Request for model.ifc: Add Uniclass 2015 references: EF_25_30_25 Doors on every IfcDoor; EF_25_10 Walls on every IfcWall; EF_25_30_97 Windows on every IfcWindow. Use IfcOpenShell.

First a look at what the model holds.

```python
import ifcopenshell

model = ifcopenshell.open("model.ifc")
print(model.schema)
print("classifications:", [c.Name for c in model.by_type("IfcClassification")])
for ifc_class in ("IfcDoor", "IfcRoof", "IfcStair", "IfcWall", "IfcWindow"):
    print(ifc_class, len(model.by_type(ifc_class)))
```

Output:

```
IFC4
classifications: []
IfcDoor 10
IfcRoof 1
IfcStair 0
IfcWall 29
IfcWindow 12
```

```python
import ifcopenshell
import ifcopenshell.api.classification

model = ifcopenshell.open("model.ifc")

system = ifcopenshell.api.classification.add_classification(model, classification="Uniclass 2015")

codes = {
    "IfcDoor": ("EF_25_30_25", "Doors"),
    "IfcWall": ("EF_25_10", "Walls"),
    "IfcWindow": ("EF_25_30_97", "Windows"),
}
for ifc_class, (code, name) in codes.items():
    products = model.by_type(ifc_class)
    ifcopenshell.api.classification.add_reference(
        model, products=products, classification=system, identification=code, name=name
    )
    print(code, len(products))

model.write("model_rev.ifc")
```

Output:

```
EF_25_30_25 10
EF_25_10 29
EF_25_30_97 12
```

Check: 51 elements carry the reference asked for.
